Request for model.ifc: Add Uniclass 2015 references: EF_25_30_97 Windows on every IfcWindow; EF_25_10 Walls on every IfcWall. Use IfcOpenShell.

First a look at what the model holds.

```python
import ifcopenshell

model = ifcopenshell.open("model.ifc")
print(model.schema)
print("classifications:", [c.Name for c in model.by_type("IfcClassification")])
for ifc_class in ("IfcDoor", "IfcRoof", "IfcStair", "IfcWall", "IfcWindow"):
    print(ifc_class, len(model.by_type(ifc_class)))
```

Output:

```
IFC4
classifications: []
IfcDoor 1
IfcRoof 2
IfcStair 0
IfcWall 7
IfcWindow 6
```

```python
import ifcopenshell
import ifcopenshell.api.classification

model = ifcopenshell.open("model.ifc")

system = ifcopenshell.api.classification.add_classification(model, classification="Uniclass 2015")

codes = {
    "IfcWindow": ("EF_25_30_97", "Windows"),
    "IfcWall": ("EF_25_10", "Walls"),
}
for ifc_class, (code, name) in codes.items():
    products = model.by_type(ifc_class)
    ifcopenshell.api.classification.add_reference(
        model, products=products, classification=system, identification=code, name=name
    )
    print(code, len(products))

model.write("model_v2.ifc")
```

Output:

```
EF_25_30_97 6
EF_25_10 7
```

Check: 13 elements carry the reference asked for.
